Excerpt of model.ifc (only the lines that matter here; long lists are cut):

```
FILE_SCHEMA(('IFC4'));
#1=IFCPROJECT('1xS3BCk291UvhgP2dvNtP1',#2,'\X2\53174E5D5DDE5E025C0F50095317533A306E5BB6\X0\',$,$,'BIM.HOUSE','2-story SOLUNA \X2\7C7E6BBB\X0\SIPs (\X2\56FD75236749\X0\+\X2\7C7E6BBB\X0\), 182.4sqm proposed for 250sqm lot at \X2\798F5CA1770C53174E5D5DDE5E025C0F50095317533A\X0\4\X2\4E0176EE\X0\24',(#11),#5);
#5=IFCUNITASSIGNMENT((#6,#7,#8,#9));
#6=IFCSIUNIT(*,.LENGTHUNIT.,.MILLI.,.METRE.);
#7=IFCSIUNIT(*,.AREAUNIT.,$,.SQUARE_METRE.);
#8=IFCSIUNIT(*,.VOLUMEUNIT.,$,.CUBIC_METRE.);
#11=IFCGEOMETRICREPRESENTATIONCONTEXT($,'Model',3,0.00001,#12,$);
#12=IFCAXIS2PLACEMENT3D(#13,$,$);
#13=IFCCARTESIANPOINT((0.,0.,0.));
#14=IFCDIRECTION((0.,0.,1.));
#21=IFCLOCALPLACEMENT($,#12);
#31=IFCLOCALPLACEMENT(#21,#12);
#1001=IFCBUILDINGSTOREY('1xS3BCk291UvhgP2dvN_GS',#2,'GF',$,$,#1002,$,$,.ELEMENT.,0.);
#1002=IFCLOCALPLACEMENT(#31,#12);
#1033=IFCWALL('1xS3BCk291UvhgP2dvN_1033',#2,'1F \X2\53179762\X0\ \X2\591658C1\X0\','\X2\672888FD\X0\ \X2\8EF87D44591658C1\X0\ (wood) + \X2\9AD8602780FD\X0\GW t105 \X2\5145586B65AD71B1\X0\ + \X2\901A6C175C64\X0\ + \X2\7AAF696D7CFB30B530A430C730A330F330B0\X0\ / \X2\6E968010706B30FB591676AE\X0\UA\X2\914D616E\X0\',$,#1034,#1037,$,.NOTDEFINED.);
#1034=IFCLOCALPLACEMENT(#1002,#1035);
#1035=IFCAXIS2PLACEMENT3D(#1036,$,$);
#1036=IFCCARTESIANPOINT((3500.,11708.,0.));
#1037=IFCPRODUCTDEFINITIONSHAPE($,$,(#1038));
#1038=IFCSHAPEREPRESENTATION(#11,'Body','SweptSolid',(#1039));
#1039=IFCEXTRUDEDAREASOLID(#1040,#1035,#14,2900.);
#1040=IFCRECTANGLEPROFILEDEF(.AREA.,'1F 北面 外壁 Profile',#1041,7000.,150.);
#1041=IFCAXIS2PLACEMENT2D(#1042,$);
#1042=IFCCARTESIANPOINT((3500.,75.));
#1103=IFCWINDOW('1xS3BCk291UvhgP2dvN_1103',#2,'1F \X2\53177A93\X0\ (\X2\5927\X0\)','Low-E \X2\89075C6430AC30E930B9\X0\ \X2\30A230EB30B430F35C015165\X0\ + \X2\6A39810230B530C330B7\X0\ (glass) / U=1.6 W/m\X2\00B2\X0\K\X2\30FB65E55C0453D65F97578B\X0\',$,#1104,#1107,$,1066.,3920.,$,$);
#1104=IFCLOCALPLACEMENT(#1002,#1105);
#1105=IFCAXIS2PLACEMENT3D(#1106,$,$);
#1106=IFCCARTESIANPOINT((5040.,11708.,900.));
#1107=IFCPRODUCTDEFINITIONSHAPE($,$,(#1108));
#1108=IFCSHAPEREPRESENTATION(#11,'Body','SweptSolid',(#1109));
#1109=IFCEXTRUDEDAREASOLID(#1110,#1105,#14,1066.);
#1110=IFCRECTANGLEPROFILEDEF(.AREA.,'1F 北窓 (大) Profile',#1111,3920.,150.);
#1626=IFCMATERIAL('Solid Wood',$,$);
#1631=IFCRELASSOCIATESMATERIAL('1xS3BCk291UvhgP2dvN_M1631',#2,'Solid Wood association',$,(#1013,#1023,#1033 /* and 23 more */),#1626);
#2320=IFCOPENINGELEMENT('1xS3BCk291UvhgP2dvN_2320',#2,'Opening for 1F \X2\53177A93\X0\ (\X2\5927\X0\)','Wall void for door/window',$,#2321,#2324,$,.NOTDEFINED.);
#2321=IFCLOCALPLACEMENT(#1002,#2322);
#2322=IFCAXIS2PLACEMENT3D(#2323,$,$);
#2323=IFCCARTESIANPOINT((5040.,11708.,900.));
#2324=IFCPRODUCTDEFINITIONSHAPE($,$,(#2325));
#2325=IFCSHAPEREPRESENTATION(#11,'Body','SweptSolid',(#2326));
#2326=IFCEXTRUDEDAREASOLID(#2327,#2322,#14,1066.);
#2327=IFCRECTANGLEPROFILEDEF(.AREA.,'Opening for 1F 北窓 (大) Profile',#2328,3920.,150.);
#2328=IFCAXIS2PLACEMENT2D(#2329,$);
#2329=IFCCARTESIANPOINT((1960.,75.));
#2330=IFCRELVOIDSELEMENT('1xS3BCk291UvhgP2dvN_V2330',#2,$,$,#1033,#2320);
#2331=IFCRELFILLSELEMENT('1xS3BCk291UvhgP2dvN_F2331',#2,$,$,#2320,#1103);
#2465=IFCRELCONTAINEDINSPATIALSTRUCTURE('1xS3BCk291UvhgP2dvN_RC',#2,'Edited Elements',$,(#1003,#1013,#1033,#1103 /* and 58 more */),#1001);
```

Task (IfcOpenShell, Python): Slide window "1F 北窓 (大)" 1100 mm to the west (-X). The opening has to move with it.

```python
import ifcopenshell
import ifcopenshell.api.geometry
import ifcopenshell.util.placement

model = ifcopenshell.open("model.ifc")

window = model.by_guid("1xS3BCk291UvhgP2dvN_1103")
opening = window.FillsVoids[0].RelatingOpeningElement
wall = opening.VoidsElements[0].RelatingBuildingElement

wall_matrix = ifcopenshell.util.placement.get_local_placement(wall.ObjectPlacement)
shift = wall_matrix[:3, 0] * -1100.0
before = ifcopenshell.util.placement.get_local_placement(window.ObjectPlacement)[:3, 3].copy()

# The window is not placed relative to its opening, so move both.
for product in (opening, window):
    matrix = ifcopenshell.util.placement.get_local_placement(product.ObjectPlacement)
    matrix[:3, 3] += shift
    ifcopenshell.api.geometry.edit_object_placement(model, product=product, matrix=matrix, is_si=False)

after = ifcopenshell.util.placement.get_local_placement(window.ObjectPlacement)[:3, 3]
print("window moved by", (after - before).round(3) + 0.0)

model.write("model-out.ifc")
```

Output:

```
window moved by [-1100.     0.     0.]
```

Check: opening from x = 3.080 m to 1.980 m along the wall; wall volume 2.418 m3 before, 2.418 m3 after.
